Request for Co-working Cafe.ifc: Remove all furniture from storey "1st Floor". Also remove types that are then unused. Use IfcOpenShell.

First a look at what the model holds.

```python
import ifcopenshell
import ifcopenshell.util.element

model = ifcopenshell.open("Co-working Cafe.ifc")
print(model.schema)
storey = next(s for s in model.by_type("IfcBuildingStorey") if s.Name == "1st Floor")
furniture = [e for e in ifcopenshell.util.element.get_decomposition(storey) if e.is_a("IfcFurnishingElement")]
seen = {}
for e in furniture:
    element_type = ifcopenshell.util.element.get_type(e)
    name = element_type.Name if element_type not in (None, e) else None
    seen[name] = seen.get(name, 0) + 1
for name, count in sorted(seen.items(), key=str):
    print(count, "x", name)
```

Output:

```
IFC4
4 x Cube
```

```python
import ifcopenshell
import ifcopenshell.api.root
import ifcopenshell.util.element

model = ifcopenshell.open("Co-working Cafe.ifc")

storey = next(s for s in model.by_type("IfcBuildingStorey") if s.Name == "1st Floor")
furniture = [e for e in ifcopenshell.util.element.get_decomposition(storey) if e.is_a("IfcFurnishingElement")]
types = {ifcopenshell.util.element.get_type(e) for e in furniture} - {None, *furniture}

for e in furniture:
    ifcopenshell.api.root.remove_product(model, product=e)
print(len(furniture), "removed")

unused = [t for t in types if not ifcopenshell.util.element.get_types(t)]
for t in unused:
    ifcopenshell.api.root.remove_product(model, product=t)
print(len(unused), "unused types removed")

model.write("Co-working Cafe_v2.ifc")
```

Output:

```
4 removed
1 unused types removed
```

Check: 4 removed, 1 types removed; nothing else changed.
